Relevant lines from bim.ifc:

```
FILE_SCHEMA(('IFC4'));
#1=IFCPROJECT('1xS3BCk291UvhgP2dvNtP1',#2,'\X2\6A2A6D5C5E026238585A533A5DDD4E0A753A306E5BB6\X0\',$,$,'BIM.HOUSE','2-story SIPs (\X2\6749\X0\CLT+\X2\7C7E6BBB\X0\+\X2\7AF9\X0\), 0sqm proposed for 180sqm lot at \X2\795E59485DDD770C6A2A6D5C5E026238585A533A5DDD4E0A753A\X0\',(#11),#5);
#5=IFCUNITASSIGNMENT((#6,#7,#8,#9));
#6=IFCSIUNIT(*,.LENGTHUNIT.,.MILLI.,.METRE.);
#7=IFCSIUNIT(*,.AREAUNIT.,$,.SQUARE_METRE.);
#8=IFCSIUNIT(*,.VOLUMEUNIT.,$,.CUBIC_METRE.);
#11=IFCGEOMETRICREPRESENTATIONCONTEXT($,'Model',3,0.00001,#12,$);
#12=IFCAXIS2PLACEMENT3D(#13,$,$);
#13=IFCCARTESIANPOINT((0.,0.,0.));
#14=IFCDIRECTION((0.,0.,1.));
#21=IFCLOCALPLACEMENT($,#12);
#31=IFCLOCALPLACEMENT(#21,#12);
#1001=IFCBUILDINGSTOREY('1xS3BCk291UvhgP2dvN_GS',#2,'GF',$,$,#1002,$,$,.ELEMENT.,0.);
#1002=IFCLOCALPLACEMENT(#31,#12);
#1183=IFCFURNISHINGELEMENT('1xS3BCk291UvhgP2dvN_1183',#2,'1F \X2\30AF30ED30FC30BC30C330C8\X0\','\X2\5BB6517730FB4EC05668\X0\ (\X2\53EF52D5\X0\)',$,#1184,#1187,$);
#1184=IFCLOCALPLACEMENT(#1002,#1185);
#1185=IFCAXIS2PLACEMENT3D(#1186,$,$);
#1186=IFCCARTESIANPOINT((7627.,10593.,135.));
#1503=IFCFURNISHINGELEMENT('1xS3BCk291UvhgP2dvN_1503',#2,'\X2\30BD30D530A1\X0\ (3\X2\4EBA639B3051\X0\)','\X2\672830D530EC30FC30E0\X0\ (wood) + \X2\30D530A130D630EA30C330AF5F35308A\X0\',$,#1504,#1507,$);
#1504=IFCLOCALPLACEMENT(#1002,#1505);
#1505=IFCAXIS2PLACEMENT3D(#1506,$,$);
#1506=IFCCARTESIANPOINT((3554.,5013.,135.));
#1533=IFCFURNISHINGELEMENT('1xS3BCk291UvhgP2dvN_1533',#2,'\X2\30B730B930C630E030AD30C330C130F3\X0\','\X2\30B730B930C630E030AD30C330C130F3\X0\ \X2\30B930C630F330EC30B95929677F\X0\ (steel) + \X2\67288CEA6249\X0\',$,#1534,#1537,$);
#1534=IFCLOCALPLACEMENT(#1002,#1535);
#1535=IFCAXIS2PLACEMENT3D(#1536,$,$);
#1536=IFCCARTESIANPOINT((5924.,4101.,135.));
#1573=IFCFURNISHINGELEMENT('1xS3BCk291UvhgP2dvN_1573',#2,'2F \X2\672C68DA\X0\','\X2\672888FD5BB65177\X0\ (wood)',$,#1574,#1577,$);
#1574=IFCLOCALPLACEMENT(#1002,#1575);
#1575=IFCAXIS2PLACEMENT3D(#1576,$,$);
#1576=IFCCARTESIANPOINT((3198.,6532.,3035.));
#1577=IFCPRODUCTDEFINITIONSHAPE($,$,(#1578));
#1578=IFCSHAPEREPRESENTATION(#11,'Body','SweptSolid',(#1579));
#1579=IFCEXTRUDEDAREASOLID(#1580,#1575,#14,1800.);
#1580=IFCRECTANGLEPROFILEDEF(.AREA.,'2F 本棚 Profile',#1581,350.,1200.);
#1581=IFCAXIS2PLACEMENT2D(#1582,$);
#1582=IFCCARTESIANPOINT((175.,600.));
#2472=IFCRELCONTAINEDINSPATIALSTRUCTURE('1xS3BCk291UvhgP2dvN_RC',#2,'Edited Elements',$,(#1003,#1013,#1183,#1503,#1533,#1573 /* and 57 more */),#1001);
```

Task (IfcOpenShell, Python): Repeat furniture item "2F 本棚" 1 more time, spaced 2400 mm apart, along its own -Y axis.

```python
import ifcopenshell
import ifcopenshell.api.geometry
import ifcopenshell.api.root
import ifcopenshell.util.element
import ifcopenshell.util.placement
import ifcopenshell.util.unit

model = ifcopenshell.open("bim.ifc")
unit_scale = ifcopenshell.util.unit.calculate_unit_scale(model)


def reuse_history(source, copy):
    """copy_class also copies each property set's owner history, people and application; keep the originals."""
    for rel in copy.IsDefinedBy:
        if rel.is_a("IfcRelDefinesByProperties") and (history := rel.RelatingPropertyDefinition.OwnerHistory):
            rel.RelatingPropertyDefinition.OwnerHistory = source.OwnerHistory
            ifcopenshell.util.element.remove_deep2(model, history)


source = model.by_guid("1xS3BCk291UvhgP2dvN_1573")
base = ifcopenshell.util.placement.get_local_placement(source.ObjectPlacement)
step = -base[:3, 1] * 2.4 / unit_scale

for i in range(1, 2):
    copy = ifcopenshell.api.root.copy_class(model, product=source)
    copy.Representation = ifcopenshell.util.element.copy_deep(
        model, source.Representation, exclude=["IfcGeometricRepresentationContext", "IfcRepresentationMap"]
    )
    reuse_history(source, copy)
    matrix = base.copy()
    matrix[:3, 3] += i * step
    print("added at", matrix[:3, 3].round(3) + 0.0)
    ifcopenshell.api.geometry.edit_object_placement(model, product=copy, matrix=matrix, is_si=False)

model.write("bim_v2.ifc")
```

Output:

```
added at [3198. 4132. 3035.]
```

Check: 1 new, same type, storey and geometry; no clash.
